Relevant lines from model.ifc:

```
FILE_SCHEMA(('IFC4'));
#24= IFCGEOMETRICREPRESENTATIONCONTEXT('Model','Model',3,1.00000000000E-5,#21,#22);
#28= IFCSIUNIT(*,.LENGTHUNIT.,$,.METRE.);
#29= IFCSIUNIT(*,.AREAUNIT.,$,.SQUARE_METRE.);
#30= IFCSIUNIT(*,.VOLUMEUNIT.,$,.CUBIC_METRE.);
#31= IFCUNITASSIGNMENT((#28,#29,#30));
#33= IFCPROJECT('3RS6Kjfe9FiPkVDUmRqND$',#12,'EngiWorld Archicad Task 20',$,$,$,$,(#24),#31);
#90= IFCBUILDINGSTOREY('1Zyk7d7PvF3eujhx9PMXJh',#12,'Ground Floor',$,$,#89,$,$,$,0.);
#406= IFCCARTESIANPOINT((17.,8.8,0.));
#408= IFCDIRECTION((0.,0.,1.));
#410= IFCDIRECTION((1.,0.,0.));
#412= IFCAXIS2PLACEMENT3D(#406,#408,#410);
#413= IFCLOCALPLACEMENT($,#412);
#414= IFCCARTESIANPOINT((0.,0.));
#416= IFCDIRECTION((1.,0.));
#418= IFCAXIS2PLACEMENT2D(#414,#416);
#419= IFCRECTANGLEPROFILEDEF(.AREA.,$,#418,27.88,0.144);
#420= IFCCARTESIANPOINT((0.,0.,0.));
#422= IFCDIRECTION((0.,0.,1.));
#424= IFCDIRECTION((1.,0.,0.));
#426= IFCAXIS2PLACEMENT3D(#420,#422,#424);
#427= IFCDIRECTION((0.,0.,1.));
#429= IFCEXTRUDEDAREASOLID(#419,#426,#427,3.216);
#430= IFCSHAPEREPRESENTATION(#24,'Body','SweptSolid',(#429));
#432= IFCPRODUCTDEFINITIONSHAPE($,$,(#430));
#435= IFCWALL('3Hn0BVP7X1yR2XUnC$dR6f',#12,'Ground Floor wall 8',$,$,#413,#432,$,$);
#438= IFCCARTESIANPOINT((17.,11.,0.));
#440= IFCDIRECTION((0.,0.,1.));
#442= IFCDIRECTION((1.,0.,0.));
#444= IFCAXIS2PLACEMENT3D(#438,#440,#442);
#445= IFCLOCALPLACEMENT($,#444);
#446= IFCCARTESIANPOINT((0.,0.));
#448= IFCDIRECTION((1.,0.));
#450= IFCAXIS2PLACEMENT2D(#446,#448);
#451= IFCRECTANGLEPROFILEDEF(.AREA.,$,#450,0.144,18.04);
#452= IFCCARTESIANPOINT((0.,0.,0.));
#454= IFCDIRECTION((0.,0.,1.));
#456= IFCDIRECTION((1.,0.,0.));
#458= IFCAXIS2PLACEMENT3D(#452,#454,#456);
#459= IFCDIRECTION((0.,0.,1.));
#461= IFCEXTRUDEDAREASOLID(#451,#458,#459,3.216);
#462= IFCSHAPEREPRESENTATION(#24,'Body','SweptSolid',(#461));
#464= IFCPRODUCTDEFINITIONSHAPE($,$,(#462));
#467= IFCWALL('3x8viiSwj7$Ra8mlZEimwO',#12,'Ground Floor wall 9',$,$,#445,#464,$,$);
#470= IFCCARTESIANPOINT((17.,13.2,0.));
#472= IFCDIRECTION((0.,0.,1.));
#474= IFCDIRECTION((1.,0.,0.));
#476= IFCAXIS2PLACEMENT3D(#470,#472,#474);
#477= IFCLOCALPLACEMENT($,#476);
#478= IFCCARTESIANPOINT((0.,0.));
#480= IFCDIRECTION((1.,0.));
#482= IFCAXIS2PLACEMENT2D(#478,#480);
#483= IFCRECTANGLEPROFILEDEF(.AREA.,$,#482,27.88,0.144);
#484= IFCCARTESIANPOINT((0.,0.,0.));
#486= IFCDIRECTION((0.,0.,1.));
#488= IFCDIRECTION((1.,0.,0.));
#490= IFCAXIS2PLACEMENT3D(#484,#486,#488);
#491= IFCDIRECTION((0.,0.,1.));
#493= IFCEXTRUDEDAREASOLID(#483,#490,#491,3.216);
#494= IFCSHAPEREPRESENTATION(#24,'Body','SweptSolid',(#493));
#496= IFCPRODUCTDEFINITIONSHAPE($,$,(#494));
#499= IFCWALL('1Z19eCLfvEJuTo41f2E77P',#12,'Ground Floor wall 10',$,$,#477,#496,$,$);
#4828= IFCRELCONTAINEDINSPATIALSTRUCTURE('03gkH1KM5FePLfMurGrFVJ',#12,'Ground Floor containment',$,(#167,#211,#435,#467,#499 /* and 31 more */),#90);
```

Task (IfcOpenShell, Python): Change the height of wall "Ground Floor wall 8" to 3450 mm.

```python
import ifcopenshell
import ifcopenshell.geom
import ifcopenshell.util.shape

model = ifcopenshell.open("model.ifc")
settings = ifcopenshell.geom.settings()


def volume(element):
    """Net volume in cubic metres, openings subtracted."""
    shape = ifcopenshell.geom.create_shape(settings, element)
    return ifcopenshell.util.shape.get_volume(shape.geometry)


wall = model.by_guid("3Hn0BVP7X1yR2XUnC$dR6f")
before = volume(wall)

body = next(r for r in wall.Representation.Representations if r.RepresentationIdentifier == "Body")
solid = body.Items[0]
old_height = solid.Depth
solid.Depth = 3.45
after = volume(wall)

print(f"height {old_height:g} -> {solid.Depth:g}, volume {before:.3f} -> {after:.3f} m3")

model.write("model_edited.ifc")
```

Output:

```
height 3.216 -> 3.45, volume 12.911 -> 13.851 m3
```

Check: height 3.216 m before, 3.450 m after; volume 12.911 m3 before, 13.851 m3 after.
